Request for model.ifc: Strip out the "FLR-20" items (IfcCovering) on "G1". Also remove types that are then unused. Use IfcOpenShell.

First a look at what the model holds.

```python
import ifcopenshell
import ifcopenshell.util.element

model = ifcopenshell.open("model.ifc")
print(model.schema)
storey = next(s for s in model.by_type("IfcBuildingStorey") if s.Name == "G1")
coverings = [e for e in ifcopenshell.util.element.get_decomposition(storey) if e.is_a("IfcCovering")]
seen = {}
for e in coverings:
    element_type = ifcopenshell.util.element.get_type(e)
    name = element_type.Name if element_type not in (None, e) else None
    seen[name] = seen.get(name, 0) + 1
for name, count in sorted(seen.items(), key=str):
    print(count, "x", name)
```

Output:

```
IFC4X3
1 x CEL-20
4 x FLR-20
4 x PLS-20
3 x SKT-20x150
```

```python
import ifcopenshell
import ifcopenshell.api.root
import ifcopenshell.util.element

model = ifcopenshell.open("model.ifc")

storey = next(s for s in model.by_type("IfcBuildingStorey") if s.Name == "G1")
coverings = [e for e in ifcopenshell.util.element.get_decomposition(storey) if e.is_a("IfcCovering")]
targets = [e for e in coverings if (t := ifcopenshell.util.element.get_type(e)) not in (None, e) and t.Name == "FLR-20"]
types = {ifcopenshell.util.element.get_type(e) for e in targets} - {None, *targets}

for e in targets:
    ifcopenshell.api.root.remove_product(model, product=e)
print(len(targets), "removed")

unused = [t for t in types if not ifcopenshell.util.element.get_types(t)]
for t in unused:
    ifcopenshell.api.root.remove_product(model, product=t)
print(len(unused), "unused types removed")

model.write("model-out.ifc")
```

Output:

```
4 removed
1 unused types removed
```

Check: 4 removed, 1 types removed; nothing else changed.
